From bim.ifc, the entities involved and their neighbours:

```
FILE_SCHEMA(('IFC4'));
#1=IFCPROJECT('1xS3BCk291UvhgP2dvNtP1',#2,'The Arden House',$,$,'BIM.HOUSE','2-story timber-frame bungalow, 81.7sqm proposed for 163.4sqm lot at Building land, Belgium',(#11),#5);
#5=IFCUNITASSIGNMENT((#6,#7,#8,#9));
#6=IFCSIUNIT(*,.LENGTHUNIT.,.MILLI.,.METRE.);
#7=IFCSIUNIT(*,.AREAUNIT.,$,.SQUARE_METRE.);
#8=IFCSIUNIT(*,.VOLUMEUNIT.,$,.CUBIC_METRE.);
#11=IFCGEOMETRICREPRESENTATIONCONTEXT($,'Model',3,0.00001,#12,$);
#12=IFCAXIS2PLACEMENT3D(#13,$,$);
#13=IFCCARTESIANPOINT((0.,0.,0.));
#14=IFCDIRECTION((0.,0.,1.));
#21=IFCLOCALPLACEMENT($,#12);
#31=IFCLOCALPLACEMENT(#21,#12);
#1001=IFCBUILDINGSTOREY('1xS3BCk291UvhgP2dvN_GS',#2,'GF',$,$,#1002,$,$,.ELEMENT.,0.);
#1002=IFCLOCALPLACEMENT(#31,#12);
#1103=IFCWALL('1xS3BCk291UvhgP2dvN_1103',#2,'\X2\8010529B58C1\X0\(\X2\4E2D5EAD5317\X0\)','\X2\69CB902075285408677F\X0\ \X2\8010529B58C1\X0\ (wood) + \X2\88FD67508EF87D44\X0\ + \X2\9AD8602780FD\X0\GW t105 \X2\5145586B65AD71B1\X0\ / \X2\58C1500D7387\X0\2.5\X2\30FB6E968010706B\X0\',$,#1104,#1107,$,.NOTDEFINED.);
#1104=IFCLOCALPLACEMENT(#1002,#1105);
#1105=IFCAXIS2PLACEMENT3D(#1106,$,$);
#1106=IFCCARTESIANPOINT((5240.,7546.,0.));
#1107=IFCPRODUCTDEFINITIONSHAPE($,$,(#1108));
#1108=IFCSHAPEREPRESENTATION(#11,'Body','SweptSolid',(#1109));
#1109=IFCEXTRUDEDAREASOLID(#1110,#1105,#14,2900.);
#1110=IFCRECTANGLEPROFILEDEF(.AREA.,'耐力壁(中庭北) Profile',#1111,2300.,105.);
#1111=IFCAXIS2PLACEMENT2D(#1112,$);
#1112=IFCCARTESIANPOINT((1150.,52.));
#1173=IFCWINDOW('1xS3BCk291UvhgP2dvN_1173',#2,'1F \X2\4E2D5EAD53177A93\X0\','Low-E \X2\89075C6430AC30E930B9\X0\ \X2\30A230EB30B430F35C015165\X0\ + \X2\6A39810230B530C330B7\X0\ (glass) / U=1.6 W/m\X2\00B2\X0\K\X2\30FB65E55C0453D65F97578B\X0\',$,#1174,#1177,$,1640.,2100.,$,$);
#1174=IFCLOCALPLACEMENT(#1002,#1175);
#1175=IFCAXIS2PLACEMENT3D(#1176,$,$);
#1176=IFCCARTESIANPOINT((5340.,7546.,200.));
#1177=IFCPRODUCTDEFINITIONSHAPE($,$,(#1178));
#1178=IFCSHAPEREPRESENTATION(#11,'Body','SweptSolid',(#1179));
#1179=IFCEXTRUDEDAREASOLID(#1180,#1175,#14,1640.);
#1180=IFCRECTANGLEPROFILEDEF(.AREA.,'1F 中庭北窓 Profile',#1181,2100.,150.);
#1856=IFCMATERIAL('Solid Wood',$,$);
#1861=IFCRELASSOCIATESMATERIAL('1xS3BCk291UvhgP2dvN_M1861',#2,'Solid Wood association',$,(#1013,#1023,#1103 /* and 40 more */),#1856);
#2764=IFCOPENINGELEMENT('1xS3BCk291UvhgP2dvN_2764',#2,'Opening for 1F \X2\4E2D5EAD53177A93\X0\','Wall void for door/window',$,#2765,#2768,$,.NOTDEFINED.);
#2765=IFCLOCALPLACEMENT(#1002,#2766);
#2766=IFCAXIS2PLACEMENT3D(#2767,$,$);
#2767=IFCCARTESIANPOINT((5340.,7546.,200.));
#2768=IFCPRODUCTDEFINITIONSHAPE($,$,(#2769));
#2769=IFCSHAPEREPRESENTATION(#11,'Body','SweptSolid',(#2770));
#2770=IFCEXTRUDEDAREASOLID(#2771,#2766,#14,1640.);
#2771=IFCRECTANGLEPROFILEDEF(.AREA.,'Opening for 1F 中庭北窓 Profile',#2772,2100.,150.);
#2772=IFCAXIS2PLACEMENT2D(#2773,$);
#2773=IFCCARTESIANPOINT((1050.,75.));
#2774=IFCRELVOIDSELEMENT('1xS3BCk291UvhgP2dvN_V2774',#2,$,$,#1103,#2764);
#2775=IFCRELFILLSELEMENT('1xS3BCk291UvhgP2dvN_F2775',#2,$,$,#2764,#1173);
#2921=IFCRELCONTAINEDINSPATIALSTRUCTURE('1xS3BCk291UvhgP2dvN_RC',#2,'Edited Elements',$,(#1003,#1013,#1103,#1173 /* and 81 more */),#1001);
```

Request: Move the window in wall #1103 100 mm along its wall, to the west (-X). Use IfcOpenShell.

```python
import ifcopenshell
import ifcopenshell.api.geometry
import ifcopenshell.util.placement
import ifcopenshell.util.unit

model = ifcopenshell.open("bim.ifc")
unit_scale = ifcopenshell.util.unit.calculate_unit_scale(model)

window = model.by_guid("1xS3BCk291UvhgP2dvN_1173")
opening = window.FillsVoids[0].RelatingOpeningElement
wall = opening.VoidsElements[0].RelatingBuildingElement

wall_matrix = ifcopenshell.util.placement.get_local_placement(wall.ObjectPlacement)
shift = wall_matrix[:3, 0] * -0.1 / unit_scale
before = ifcopenshell.util.placement.get_local_placement(window.ObjectPlacement)[:3, 3].copy()

# The window is not placed relative to its opening, so move both.
for product in (opening, window):
    matrix = ifcopenshell.util.placement.get_local_placement(product.ObjectPlacement)
    matrix[:3, 3] += shift
    ifcopenshell.api.geometry.edit_object_placement(model, product=product, matrix=matrix, is_si=False)

after = ifcopenshell.util.placement.get_local_placement(window.ObjectPlacement)[:3, 3]
print("window moved by", (after - before).round(3) + 0.0)

model.write("bim-out.ifc")
```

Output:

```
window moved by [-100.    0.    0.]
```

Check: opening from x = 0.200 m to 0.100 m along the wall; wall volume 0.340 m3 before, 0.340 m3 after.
